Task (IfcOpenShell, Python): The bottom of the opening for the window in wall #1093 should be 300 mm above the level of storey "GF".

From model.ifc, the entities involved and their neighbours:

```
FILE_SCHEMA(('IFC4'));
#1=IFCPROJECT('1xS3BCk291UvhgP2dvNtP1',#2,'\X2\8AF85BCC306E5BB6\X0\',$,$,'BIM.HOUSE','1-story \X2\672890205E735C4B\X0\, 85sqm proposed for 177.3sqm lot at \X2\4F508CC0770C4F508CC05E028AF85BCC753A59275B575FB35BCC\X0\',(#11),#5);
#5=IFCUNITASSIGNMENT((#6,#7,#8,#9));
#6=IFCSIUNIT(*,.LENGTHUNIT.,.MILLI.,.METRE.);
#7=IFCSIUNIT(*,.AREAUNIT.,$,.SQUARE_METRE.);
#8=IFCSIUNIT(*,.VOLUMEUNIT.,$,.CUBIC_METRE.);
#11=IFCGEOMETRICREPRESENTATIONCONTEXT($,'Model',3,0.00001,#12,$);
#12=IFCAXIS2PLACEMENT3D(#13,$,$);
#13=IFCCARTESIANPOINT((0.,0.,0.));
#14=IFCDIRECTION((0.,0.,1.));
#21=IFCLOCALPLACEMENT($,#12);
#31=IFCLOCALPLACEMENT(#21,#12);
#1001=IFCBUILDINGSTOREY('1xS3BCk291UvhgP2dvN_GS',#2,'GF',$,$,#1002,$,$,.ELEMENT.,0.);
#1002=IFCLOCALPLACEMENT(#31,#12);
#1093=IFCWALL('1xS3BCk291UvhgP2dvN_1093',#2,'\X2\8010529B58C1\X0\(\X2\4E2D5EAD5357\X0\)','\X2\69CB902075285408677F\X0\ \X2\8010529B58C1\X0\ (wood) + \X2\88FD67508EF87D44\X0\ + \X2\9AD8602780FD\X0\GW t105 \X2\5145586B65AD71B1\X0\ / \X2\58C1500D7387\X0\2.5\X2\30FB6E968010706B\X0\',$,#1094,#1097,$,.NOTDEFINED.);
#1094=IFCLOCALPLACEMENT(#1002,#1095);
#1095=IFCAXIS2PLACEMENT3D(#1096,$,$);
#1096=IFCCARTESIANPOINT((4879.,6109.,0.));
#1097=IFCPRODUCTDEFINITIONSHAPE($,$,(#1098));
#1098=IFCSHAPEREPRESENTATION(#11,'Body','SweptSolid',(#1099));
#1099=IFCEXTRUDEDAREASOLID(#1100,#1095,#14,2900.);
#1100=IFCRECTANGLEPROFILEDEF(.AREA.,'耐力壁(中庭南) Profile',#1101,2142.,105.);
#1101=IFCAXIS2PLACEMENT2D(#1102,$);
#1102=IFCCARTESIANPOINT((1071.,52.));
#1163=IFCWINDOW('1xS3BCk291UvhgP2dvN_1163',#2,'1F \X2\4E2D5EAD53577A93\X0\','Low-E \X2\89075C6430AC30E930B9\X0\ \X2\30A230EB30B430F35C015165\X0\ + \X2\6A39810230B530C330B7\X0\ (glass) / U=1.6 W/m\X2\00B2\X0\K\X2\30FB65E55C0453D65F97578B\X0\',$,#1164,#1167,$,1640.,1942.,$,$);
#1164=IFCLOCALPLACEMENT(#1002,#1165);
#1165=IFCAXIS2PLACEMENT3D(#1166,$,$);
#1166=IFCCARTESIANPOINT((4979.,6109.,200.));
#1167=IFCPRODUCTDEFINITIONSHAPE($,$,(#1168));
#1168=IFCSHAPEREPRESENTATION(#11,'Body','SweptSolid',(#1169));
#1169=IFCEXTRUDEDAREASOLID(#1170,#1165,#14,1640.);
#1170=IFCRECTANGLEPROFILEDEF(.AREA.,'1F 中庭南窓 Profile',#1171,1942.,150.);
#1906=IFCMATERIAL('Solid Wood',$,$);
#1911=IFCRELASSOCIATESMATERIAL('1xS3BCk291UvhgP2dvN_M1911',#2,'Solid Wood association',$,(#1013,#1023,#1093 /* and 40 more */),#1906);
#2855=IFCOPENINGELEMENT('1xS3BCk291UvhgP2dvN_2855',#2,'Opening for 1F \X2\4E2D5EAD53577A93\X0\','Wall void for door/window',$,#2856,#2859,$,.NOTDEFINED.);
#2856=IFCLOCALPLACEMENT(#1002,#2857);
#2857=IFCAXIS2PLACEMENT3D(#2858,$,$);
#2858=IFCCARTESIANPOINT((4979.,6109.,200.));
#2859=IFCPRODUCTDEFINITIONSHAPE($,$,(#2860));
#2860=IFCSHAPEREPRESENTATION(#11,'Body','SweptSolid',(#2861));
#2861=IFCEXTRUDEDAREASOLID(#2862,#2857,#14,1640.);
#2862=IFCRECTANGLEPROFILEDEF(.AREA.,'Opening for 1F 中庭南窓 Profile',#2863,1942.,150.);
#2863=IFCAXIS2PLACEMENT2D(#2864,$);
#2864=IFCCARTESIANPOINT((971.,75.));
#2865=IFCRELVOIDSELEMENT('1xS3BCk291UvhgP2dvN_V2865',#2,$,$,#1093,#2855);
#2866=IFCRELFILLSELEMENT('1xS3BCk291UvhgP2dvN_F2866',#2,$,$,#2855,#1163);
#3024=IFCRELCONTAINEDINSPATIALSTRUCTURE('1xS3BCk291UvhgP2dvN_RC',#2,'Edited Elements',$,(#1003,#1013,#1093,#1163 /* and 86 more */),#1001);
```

```python
import numpy as np
import ifcopenshell
import ifcopenshell.api.geometry
import ifcopenshell.geom
import ifcopenshell.util.element
import ifcopenshell.util.placement
import ifcopenshell.util.shape
import ifcopenshell.util.unit

model = ifcopenshell.open("model.ifc")
unit_scale = ifcopenshell.util.unit.calculate_unit_scale(model)

window = model.by_guid("1xS3BCk291UvhgP2dvN_1163")
opening = window.FillsVoids[0].RelatingOpeningElement
storey = ifcopenshell.util.element.get_container(window, ifc_class="IfcBuildingStorey")
level = ifcopenshell.util.placement.get_local_placement(storey.ObjectPlacement)[2, 3]

# The opening's origin need not be at the sill, so measure its lowest point.
shape = ifcopenshell.geom.create_shape(ifcopenshell.geom.settings(), opening)
bottom = ifcopenshell.util.shape.get_shape_bottom_elevation(shape, shape.geometry) / unit_scale
dz = level + 300.0 - bottom

shift = np.array([0.0, 0.0, dz])
# The window is not placed relative to its opening, so move both.
for product in (opening, window):
    matrix = ifcopenshell.util.placement.get_local_placement(product.ObjectPlacement)
    matrix[:3, 3] += shift
    ifcopenshell.api.geometry.edit_object_placement(model, product=product, matrix=matrix, is_si=False)

print(f"moved by {dz * unit_scale:+.3f} m")

model.write("model_updated.ifc")
```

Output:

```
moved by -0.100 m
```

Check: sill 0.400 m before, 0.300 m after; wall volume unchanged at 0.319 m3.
